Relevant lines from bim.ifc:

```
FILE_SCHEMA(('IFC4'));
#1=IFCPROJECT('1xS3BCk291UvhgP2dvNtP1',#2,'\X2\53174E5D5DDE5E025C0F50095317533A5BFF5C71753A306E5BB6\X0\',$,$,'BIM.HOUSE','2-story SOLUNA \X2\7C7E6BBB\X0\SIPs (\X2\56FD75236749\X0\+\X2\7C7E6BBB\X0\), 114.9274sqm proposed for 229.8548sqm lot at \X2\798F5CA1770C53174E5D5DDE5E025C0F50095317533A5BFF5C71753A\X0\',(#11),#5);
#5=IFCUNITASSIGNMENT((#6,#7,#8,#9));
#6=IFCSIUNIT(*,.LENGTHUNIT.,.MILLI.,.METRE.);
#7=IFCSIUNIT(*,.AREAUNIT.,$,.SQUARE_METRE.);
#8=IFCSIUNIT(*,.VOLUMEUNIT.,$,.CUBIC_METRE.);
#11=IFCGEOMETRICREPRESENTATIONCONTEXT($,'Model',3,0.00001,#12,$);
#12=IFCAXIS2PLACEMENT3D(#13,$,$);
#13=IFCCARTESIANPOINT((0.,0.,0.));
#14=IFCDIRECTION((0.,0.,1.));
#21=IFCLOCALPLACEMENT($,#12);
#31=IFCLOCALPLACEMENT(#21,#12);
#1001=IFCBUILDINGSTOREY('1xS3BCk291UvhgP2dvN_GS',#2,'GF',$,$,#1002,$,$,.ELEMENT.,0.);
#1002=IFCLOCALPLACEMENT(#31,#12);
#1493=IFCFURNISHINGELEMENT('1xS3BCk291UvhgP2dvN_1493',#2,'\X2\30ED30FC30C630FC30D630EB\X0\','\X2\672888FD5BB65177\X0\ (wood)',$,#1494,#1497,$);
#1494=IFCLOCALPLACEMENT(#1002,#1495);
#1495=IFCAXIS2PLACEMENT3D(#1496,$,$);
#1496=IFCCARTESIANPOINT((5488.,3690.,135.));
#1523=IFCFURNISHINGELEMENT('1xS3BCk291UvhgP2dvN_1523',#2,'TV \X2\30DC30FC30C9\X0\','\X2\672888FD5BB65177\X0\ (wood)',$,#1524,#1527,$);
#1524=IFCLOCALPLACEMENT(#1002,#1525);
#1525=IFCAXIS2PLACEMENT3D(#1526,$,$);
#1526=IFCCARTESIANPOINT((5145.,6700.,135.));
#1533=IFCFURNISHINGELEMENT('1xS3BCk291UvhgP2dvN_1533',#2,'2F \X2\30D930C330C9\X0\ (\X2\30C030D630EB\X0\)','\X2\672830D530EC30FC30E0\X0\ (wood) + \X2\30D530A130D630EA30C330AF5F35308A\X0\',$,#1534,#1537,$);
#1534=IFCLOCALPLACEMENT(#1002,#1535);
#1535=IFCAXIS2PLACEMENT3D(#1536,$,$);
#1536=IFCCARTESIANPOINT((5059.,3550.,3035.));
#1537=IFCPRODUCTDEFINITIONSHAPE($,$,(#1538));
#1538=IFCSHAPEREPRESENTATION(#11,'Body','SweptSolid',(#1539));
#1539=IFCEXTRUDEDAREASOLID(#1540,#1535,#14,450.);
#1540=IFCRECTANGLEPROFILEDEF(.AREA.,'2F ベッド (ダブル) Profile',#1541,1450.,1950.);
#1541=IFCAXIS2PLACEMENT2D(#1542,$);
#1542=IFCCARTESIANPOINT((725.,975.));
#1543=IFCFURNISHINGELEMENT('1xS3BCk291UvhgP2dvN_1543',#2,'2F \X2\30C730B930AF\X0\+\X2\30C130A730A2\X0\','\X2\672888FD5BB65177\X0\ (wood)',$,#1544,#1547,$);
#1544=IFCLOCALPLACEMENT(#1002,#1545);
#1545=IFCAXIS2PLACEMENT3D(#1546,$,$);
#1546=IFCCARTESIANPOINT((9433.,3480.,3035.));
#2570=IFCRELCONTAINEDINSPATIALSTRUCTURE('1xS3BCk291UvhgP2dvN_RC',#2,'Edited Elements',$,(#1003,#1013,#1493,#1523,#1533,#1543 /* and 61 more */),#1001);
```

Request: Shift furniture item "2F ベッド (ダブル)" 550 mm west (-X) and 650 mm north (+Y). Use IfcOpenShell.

```python
import ifcopenshell
import ifcopenshell.api.geometry
import ifcopenshell.util.placement
import ifcopenshell.util.unit

model = ifcopenshell.open("bim.ifc")
unit_scale = ifcopenshell.util.unit.calculate_unit_scale(model)

item = model.by_guid("1xS3BCk291UvhgP2dvN_1533")
matrix = ifcopenshell.util.placement.get_local_placement(item.ObjectPlacement)
matrix[0, 3] -= 0.55 / unit_scale
matrix[1, 3] += 0.65 / unit_scale
ifcopenshell.api.geometry.edit_object_placement(model, product=item, matrix=matrix, is_si=False)

print(ifcopenshell.util.placement.get_local_placement(item.ObjectPlacement).round(3) + 0.0)

model.write("bim_v2.ifc")
```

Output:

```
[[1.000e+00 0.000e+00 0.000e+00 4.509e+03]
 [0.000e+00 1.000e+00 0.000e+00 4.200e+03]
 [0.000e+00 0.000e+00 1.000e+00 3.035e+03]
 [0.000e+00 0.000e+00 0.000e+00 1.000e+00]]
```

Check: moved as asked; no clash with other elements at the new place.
